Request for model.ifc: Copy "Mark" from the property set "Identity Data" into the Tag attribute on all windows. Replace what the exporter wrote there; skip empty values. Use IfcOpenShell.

First a look at what the model holds.

```python
import ifcopenshell
import ifcopenshell.util.element

model = ifcopenshell.open("model.ifc")
print(model.schema)
windows = model.by_type("IfcWindow")
print(len(windows), "windows")
for e in windows[:8]:
    source = ifcopenshell.util.element.get_pset(e, "Identity Data", "Mark")
    target = e.Tag
    print(e.id(), repr(source), repr(target), sep=" | ")
```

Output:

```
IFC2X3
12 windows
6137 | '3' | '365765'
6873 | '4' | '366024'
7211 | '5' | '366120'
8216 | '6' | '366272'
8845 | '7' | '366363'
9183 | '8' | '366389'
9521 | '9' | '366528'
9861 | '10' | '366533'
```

```python
import ifcopenshell
import ifcopenshell.util.element

model = ifcopenshell.open("model.ifc")

count = 0
for e in model.by_type("IfcWindow"):
    value = ifcopenshell.util.element.get_pset(e, "Identity Data", "Mark")
    current = e.Tag
    if not value or not value.strip() or current == value:
        continue
    e.Tag = value
    count += 1

print(count, "windows updated")

model.write("model_rev.ifc")
```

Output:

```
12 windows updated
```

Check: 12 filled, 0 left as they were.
